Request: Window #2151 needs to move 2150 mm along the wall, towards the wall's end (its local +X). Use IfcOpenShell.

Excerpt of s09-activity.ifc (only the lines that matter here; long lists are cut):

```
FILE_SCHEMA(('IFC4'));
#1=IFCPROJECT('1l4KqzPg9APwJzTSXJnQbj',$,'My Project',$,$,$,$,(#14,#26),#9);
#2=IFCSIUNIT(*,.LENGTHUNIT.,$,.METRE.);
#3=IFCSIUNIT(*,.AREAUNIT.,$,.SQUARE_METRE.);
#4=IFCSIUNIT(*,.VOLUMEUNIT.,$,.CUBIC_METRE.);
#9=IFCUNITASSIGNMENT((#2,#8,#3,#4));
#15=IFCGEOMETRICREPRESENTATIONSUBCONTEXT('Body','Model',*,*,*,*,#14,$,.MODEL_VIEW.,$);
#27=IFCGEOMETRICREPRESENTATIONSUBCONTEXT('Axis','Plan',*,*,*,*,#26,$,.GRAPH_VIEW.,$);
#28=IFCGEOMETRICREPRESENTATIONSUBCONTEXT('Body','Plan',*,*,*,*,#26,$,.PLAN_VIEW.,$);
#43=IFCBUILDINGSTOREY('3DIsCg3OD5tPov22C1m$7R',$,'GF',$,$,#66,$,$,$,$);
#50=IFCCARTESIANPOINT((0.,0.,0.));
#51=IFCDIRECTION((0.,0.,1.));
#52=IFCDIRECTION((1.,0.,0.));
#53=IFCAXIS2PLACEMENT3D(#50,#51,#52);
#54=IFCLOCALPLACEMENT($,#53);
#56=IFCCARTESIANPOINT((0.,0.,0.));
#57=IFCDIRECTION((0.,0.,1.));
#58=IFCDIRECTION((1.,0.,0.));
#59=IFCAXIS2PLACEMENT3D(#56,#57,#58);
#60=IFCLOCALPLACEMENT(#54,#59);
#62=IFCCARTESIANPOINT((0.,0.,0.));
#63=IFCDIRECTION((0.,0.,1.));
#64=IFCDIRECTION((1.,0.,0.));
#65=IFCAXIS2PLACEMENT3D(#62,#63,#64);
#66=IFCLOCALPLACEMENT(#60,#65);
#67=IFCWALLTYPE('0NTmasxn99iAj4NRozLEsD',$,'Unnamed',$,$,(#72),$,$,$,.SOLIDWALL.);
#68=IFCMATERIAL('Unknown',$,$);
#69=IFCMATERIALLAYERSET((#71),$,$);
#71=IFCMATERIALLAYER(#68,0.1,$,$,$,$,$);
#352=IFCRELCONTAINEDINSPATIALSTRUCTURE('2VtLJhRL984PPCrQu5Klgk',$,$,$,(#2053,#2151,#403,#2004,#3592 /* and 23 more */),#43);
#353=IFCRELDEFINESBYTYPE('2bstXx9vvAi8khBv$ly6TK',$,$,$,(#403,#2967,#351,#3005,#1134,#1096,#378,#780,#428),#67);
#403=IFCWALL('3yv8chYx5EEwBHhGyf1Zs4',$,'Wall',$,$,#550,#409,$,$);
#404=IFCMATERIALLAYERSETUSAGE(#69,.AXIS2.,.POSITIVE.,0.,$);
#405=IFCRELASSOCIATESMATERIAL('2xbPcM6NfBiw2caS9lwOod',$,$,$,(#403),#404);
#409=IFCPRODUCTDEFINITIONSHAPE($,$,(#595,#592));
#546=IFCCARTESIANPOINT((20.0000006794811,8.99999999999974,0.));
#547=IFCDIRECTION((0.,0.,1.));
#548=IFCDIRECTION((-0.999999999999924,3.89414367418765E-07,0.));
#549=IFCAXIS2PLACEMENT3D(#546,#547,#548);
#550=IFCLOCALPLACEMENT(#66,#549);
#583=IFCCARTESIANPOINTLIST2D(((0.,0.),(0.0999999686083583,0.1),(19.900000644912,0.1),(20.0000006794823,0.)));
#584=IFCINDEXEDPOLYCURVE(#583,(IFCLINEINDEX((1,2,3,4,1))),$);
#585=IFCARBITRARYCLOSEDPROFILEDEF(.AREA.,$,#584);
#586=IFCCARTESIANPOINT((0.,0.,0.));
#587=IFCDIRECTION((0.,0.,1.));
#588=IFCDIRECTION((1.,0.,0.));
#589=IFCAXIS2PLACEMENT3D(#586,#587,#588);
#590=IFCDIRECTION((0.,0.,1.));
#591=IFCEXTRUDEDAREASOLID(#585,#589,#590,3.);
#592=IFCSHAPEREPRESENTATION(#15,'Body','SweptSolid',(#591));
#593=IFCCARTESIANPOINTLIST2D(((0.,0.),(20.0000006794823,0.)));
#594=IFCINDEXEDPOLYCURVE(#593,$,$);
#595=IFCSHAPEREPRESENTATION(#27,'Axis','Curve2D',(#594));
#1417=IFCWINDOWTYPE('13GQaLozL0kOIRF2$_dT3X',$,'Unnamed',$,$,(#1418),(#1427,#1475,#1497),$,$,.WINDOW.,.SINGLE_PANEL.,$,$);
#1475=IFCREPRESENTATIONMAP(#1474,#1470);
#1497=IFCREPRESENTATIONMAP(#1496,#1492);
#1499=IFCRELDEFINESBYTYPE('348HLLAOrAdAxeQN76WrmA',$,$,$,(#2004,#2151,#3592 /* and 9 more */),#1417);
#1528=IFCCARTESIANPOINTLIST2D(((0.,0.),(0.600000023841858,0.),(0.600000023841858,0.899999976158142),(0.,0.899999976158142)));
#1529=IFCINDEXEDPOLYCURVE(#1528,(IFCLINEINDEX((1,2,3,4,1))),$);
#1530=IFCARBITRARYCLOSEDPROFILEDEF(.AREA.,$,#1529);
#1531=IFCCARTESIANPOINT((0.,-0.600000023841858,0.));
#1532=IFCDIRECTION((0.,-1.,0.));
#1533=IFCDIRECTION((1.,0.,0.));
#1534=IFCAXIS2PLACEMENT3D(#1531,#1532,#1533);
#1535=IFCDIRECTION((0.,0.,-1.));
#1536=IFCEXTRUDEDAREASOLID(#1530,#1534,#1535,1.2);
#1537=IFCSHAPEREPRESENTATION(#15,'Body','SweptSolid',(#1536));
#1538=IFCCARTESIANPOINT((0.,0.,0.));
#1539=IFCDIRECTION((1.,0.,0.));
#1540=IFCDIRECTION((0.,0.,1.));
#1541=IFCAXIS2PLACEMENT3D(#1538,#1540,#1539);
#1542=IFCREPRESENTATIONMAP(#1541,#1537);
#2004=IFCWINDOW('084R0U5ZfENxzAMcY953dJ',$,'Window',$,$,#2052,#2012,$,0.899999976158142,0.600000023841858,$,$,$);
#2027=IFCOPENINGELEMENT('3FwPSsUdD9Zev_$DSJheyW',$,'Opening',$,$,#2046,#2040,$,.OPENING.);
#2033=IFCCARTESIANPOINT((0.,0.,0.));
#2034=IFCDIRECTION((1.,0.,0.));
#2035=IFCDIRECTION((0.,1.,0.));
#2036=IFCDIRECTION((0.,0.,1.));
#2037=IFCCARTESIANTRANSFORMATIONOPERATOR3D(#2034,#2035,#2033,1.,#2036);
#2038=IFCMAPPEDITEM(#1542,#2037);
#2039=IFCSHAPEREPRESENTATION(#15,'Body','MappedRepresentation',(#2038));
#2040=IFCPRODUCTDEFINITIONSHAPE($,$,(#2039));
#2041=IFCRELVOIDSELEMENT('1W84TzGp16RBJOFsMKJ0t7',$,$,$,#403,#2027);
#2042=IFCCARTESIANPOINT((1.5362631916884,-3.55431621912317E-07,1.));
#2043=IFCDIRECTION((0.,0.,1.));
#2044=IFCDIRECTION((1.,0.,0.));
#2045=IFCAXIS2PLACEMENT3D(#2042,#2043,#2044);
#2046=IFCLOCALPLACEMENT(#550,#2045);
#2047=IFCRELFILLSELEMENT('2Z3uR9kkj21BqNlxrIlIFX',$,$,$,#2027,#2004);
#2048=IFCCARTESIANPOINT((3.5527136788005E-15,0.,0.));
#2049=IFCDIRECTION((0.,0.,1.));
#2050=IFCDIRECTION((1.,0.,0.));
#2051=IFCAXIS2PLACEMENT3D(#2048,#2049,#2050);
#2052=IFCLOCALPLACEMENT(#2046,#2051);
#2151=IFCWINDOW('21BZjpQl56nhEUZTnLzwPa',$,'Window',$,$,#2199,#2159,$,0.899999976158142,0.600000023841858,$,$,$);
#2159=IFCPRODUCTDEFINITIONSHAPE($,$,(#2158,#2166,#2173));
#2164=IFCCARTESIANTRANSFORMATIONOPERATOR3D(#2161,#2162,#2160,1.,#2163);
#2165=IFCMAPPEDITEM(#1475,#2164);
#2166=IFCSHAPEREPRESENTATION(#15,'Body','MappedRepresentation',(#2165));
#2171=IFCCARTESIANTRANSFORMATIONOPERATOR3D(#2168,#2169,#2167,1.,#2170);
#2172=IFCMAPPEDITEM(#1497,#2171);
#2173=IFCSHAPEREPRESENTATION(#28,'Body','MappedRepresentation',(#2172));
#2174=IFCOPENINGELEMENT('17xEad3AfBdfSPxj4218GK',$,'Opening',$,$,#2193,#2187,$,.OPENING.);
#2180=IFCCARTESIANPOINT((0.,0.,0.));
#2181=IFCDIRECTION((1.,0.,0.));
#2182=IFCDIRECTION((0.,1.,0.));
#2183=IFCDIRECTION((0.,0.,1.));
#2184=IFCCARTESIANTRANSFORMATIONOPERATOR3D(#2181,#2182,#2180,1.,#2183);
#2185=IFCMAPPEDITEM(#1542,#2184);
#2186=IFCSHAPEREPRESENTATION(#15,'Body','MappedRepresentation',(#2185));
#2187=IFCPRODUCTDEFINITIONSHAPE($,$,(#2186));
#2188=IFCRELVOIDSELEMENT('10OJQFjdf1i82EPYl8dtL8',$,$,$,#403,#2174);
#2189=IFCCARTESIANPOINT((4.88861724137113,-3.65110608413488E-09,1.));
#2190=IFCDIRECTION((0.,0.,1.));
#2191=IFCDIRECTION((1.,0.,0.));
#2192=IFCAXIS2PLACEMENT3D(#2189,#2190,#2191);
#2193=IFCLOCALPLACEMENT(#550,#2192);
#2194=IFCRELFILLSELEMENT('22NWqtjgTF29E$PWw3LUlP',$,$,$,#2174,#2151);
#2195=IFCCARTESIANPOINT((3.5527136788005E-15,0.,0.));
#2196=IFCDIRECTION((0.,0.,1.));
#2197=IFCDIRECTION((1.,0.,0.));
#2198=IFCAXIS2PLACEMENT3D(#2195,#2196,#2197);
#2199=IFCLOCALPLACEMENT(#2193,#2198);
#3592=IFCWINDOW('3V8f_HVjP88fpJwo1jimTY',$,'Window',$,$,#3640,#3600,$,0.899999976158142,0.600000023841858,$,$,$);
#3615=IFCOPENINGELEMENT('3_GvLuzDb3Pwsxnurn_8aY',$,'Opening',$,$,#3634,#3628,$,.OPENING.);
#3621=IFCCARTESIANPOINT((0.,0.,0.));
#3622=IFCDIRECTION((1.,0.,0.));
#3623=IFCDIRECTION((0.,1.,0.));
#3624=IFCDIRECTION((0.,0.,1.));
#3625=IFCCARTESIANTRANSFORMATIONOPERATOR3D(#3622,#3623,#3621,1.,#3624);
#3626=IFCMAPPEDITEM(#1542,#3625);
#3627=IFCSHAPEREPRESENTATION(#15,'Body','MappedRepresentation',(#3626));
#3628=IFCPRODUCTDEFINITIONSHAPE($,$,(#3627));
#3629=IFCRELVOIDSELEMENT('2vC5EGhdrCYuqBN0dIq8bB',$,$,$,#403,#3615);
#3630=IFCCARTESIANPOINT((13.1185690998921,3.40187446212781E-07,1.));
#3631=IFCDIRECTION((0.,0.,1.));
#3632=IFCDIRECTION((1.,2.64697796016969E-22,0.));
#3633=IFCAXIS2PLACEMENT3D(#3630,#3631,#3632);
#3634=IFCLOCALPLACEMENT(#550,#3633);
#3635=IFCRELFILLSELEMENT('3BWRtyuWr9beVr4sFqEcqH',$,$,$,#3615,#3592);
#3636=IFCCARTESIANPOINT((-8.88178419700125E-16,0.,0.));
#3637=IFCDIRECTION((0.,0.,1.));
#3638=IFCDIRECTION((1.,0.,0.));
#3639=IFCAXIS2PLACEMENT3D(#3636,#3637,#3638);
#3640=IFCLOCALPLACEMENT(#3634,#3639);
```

```python
import ifcopenshell
import ifcopenshell.api.geometry
import ifcopenshell.util.placement
import ifcopenshell.util.unit

model = ifcopenshell.open("s09-activity.ifc")
unit_scale = ifcopenshell.util.unit.calculate_unit_scale(model)

window = model.by_guid("21BZjpQl56nhEUZTnLzwPa")
opening = window.FillsVoids[0].RelatingOpeningElement
wall = opening.VoidsElements[0].RelatingBuildingElement

wall_matrix = ifcopenshell.util.placement.get_local_placement(wall.ObjectPlacement)
shift = wall_matrix[:3, 0] * 2.15 / unit_scale
before = ifcopenshell.util.placement.get_local_placement(window.ObjectPlacement)[:3, 3].copy()

# The window is placed relative to its opening, so it follows when the opening moves.
matrix = ifcopenshell.util.placement.get_local_placement(opening.ObjectPlacement)
matrix[:3, 3] += shift
ifcopenshell.api.geometry.edit_object_placement(
    model, product=opening, matrix=matrix, is_si=False, should_transform_children=True
)

after = ifcopenshell.util.placement.get_local_placement(window.ObjectPlacement)[:3, 3]
print("window moved by", (after - before).round(3) + 0.0)

model.write("s09-activity-out.ifc")
```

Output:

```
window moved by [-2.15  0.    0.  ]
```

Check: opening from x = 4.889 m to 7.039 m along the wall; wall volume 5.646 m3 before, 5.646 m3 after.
